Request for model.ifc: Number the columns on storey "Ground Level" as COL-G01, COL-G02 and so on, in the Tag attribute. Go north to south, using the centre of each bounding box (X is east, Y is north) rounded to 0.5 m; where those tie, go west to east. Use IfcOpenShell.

First a look at what the model holds.

```python
import ifcopenshell
import ifcopenshell.util.element
import ifcopenshell.util.placement

model = ifcopenshell.open("model.ifc")
print(model.schema)
storey = next(s for s in model.by_type("IfcBuildingStorey") if s.Name == "Ground Level")
columns = [e for e in ifcopenshell.util.element.get_decomposition(storey) if e.is_a("IfcColumn")]
for e in sorted(columns, key=lambda e: e.id()):
    origin = ifcopenshell.util.placement.get_local_placement(e.ObjectPlacement)[:3, 3]
    print(e.id(), e.Tag, e.Name, origin.round(2) + 0.0, sep=" | ")
```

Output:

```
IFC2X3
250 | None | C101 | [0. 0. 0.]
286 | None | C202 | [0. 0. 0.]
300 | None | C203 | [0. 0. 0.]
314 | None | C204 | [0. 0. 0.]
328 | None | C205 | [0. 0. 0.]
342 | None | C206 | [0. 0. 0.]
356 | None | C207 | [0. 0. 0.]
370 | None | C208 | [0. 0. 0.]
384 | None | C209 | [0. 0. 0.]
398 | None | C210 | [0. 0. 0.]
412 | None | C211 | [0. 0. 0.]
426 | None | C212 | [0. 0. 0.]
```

```python
import ifcopenshell
import ifcopenshell.geom
import ifcopenshell.util.element
import ifcopenshell.util.shape

model = ifcopenshell.open("model.ifc")
settings = ifcopenshell.geom.settings()
settings.set("use-world-coords", True)


def centre(element):
    shape = ifcopenshell.geom.create_shape(settings, element)
    return ifcopenshell.util.shape.get_bbox_centroid(shape.geometry)


storey = next(s for s in model.by_type("IfcBuildingStorey") if s.Name == "Ground Level")
columns = [e for e in ifcopenshell.util.element.get_decomposition(storey) if e.is_a("IfcColumn")]

# Insertion points can sit at a corner or the storey origin, so sort by the geometry (in metres).
centres = {e: centre(e) for e in columns}
columns.sort(key=lambda e: (-round(centres[e][1] / 0.5), centres[e][0]))

for i, e in enumerate(columns, start=1):
    number = f"COL-G{i:02d}"
    e.Tag = number
    print(e.id(), number)

model.write("model-out.ifc")
```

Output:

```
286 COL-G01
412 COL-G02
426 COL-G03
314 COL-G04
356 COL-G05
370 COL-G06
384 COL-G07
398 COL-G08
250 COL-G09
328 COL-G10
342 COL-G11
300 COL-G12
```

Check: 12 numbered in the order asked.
